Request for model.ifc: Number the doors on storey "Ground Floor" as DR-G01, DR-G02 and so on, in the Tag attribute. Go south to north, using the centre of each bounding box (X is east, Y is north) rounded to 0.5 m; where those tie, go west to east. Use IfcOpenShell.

First a look at what the model holds.

```python
import ifcopenshell
import ifcopenshell.util.element
import ifcopenshell.util.placement

model = ifcopenshell.open("model.ifc")
print(model.schema)
storey = next(s for s in model.by_type("IfcBuildingStorey") if s.Name == "Ground Floor")
doors = [e for e in ifcopenshell.util.element.get_decomposition(storey) if e.is_a("IfcDoor")]
for e in sorted(doors, key=lambda e: e.id()):
    origin = ifcopenshell.util.placement.get_local_placement(e.ObjectPlacement)[:3, 3]
    print(e.id(), e.Tag, e.Name, origin.round(2) + 0.0, sep=" | ")
```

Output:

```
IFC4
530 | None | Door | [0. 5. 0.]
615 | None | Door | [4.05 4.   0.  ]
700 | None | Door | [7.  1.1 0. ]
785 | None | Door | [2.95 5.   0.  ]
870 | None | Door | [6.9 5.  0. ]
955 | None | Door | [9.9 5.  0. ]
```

```python
import ifcopenshell
import ifcopenshell.geom
import ifcopenshell.util.element
import ifcopenshell.util.shape

model = ifcopenshell.open("model.ifc")
settings = ifcopenshell.geom.settings()
settings.set("use-world-coords", True)


def centre(element):
    shape = ifcopenshell.geom.create_shape(settings, element)
    return ifcopenshell.util.shape.get_bbox_centroid(shape.geometry)


storey = next(s for s in model.by_type("IfcBuildingStorey") if s.Name == "Ground Floor")
doors = [e for e in ifcopenshell.util.element.get_decomposition(storey) if e.is_a("IfcDoor")]

# Insertion points can sit at a corner or the storey origin, so sort by the geometry (in metres).
centres = {e: centre(e) for e in doors}
doors.sort(key=lambda e: (round(centres[e][1] / 0.5), centres[e][0]))

for i, e in enumerate(doors, start=1):
    number = f"DR-G{i:02d}"
    e.Tag = number
    print(e.id(), number)

model.write("model-out.ifc")
```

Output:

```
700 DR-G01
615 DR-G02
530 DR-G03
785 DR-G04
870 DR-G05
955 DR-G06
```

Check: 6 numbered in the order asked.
